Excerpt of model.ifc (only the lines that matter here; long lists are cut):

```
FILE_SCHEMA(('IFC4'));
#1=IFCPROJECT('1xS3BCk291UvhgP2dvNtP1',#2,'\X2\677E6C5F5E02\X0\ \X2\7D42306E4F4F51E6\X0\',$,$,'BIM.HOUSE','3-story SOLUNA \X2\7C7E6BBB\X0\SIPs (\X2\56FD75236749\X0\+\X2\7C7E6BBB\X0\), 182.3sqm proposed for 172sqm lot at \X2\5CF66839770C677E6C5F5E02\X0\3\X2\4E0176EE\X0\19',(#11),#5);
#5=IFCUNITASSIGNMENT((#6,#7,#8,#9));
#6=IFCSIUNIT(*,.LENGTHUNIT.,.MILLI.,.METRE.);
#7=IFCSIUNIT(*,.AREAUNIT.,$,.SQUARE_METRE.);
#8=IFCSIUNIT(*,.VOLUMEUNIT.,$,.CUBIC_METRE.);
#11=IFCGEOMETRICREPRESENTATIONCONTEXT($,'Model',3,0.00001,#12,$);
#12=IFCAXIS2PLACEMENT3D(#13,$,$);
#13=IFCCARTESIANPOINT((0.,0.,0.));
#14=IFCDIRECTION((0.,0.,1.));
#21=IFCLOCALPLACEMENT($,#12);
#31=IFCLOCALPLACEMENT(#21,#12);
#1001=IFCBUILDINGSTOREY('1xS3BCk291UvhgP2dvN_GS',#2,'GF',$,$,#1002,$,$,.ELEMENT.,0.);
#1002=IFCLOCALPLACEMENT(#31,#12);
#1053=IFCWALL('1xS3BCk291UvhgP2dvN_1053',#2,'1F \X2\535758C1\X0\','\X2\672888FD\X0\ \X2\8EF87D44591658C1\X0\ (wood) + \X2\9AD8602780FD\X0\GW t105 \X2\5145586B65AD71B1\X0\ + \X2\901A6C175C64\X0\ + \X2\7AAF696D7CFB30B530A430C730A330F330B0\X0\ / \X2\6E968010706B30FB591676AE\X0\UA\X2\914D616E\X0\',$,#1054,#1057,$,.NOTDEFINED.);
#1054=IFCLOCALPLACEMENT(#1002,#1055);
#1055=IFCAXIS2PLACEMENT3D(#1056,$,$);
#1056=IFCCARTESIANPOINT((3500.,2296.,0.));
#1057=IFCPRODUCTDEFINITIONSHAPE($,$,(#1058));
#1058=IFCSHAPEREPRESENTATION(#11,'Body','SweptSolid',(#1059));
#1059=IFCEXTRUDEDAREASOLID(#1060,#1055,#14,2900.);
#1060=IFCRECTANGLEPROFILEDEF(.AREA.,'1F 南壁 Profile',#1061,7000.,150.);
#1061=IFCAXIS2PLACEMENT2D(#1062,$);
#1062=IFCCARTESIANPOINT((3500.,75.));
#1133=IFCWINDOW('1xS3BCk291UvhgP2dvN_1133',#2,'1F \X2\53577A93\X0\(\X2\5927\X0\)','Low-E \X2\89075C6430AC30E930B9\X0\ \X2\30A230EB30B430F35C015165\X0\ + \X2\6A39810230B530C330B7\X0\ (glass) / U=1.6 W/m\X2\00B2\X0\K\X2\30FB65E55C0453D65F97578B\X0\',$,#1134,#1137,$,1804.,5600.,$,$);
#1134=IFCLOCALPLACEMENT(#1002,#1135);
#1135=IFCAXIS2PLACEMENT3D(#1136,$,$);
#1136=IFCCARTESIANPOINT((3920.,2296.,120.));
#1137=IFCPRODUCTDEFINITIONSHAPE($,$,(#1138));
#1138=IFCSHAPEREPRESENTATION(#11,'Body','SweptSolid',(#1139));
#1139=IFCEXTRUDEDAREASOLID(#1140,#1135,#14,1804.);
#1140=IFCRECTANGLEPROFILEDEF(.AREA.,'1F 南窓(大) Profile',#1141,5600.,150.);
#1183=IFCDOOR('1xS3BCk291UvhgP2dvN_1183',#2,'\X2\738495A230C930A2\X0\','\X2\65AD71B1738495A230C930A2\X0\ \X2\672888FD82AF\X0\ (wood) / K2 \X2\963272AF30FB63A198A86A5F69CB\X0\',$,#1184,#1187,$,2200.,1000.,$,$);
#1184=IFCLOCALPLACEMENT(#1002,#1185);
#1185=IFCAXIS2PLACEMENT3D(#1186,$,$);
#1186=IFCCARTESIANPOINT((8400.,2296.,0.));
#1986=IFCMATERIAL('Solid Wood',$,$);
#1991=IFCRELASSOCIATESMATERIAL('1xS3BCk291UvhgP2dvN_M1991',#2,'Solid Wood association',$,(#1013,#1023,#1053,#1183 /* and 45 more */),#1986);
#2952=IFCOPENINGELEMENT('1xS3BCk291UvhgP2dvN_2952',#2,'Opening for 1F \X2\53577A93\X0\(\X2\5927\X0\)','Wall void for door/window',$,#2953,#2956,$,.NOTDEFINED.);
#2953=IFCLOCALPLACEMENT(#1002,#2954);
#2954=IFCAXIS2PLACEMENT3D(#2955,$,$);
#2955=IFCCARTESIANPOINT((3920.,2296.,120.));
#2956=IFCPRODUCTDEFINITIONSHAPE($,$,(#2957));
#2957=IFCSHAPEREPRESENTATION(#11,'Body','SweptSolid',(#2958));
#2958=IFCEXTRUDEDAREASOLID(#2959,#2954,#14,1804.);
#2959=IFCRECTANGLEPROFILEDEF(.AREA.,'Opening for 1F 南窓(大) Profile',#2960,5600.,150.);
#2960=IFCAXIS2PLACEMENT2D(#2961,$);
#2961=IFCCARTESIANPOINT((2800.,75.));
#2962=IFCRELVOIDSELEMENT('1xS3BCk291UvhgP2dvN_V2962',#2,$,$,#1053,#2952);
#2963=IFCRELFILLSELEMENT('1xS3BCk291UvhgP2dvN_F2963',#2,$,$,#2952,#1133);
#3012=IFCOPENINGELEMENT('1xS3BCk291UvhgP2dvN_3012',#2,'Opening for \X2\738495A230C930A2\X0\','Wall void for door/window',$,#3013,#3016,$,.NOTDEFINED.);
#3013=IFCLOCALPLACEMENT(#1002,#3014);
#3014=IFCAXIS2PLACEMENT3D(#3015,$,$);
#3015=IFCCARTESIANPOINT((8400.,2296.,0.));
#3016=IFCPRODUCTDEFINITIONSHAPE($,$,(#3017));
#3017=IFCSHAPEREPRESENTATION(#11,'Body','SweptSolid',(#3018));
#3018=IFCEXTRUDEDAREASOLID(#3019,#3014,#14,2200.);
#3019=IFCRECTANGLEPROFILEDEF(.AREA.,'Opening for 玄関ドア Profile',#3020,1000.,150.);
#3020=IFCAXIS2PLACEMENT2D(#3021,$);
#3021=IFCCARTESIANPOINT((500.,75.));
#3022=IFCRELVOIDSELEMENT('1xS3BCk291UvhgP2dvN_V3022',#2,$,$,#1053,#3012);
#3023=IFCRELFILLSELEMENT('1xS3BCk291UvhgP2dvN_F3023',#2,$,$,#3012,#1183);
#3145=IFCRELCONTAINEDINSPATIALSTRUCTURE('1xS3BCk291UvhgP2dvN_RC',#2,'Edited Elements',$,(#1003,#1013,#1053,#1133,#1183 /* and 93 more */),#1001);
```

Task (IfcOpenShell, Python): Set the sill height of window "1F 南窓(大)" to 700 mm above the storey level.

```python
import numpy as np
import ifcopenshell
import ifcopenshell.api.geometry
import ifcopenshell.geom
import ifcopenshell.util.element
import ifcopenshell.util.placement
import ifcopenshell.util.shape
import ifcopenshell.util.unit

model = ifcopenshell.open("model.ifc")
unit_scale = ifcopenshell.util.unit.calculate_unit_scale(model)

window = model.by_guid("1xS3BCk291UvhgP2dvN_1133")
opening = window.FillsVoids[0].RelatingOpeningElement
storey = ifcopenshell.util.element.get_container(window, ifc_class="IfcBuildingStorey")
level = ifcopenshell.util.placement.get_local_placement(storey.ObjectPlacement)[2, 3]

# The opening's origin need not be at the sill, so measure its lowest point.
shape = ifcopenshell.geom.create_shape(ifcopenshell.geom.settings(), opening)
bottom = ifcopenshell.util.shape.get_shape_bottom_elevation(shape, shape.geometry) / unit_scale
dz = level + 0.7 / unit_scale - bottom

shift = np.array([0.0, 0.0, dz])
# The window is not placed relative to its opening, so move both.
for product in (opening, window):
    matrix = ifcopenshell.util.placement.get_local_placement(product.ObjectPlacement)
    matrix[:3, 3] += shift
    ifcopenshell.api.geometry.edit_object_placement(model, product=product, matrix=matrix, is_si=False)

print(f"moved by {dz * unit_scale:+.3f} m")

model.write("model_updated.ifc")
```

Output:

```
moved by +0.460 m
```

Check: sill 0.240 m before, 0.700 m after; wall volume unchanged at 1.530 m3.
